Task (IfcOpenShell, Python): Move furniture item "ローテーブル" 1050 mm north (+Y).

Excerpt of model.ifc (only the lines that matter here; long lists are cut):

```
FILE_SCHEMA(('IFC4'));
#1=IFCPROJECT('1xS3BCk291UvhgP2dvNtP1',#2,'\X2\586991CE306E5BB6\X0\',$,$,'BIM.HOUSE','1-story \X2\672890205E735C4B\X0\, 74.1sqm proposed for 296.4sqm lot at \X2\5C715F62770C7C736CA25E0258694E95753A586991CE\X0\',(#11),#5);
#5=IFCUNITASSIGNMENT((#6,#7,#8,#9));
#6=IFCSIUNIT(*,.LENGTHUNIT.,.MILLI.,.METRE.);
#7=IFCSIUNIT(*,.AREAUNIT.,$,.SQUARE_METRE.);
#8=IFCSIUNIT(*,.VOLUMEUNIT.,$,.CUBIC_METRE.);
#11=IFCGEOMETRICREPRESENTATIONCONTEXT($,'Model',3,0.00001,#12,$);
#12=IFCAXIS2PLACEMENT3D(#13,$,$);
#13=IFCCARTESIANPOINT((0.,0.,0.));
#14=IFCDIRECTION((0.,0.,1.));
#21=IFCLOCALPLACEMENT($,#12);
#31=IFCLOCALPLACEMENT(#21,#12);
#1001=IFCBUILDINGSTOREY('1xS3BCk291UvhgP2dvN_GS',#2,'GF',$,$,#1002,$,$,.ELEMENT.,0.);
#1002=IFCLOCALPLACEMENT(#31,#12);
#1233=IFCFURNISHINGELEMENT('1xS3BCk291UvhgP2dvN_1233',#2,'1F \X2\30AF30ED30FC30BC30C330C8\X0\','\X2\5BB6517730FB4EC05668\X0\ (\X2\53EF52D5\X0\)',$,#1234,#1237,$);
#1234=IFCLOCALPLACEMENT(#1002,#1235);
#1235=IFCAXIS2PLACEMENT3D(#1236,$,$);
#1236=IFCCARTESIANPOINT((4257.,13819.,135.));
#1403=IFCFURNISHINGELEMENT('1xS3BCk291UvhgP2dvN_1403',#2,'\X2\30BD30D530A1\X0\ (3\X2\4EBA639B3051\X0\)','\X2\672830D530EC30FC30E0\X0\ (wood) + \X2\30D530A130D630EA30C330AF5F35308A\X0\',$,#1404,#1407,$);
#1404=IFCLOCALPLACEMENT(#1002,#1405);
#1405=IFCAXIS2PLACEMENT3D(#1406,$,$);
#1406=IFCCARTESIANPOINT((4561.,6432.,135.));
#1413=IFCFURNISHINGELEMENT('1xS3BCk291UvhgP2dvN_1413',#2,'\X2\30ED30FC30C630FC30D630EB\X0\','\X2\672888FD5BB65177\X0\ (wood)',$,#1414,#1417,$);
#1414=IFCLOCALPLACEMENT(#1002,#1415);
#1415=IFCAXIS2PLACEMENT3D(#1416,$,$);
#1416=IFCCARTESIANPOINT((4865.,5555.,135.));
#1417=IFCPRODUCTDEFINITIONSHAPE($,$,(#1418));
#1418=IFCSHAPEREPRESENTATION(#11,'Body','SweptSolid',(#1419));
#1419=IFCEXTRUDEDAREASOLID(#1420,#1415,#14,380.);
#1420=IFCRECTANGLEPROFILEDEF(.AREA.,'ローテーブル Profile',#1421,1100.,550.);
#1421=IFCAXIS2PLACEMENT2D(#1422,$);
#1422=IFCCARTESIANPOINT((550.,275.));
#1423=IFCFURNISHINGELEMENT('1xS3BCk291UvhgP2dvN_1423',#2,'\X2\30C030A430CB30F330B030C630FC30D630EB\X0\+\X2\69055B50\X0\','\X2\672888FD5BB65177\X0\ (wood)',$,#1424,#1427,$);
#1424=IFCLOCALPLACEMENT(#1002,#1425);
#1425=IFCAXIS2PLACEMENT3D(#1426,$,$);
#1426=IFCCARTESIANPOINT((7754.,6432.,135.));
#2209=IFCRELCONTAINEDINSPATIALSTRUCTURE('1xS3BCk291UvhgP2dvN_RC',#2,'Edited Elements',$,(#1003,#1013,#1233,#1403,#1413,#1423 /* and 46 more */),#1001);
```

```python
import ifcopenshell
import ifcopenshell.api.geometry
import ifcopenshell.util.placement
import ifcopenshell.util.unit

model = ifcopenshell.open("model.ifc")
unit_scale = ifcopenshell.util.unit.calculate_unit_scale(model)

item = model.by_guid("1xS3BCk291UvhgP2dvN_1413")
matrix = ifcopenshell.util.placement.get_local_placement(item.ObjectPlacement)
matrix[1, 3] += 1.05 / unit_scale
ifcopenshell.api.geometry.edit_object_placement(model, product=item, matrix=matrix, is_si=False)

print(ifcopenshell.util.placement.get_local_placement(item.ObjectPlacement).round(3) + 0.0)

model.write("model_edited.ifc")
```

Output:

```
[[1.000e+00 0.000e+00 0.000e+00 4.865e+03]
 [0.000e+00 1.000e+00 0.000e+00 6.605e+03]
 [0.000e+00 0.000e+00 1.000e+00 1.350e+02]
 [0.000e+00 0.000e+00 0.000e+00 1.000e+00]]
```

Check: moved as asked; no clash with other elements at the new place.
